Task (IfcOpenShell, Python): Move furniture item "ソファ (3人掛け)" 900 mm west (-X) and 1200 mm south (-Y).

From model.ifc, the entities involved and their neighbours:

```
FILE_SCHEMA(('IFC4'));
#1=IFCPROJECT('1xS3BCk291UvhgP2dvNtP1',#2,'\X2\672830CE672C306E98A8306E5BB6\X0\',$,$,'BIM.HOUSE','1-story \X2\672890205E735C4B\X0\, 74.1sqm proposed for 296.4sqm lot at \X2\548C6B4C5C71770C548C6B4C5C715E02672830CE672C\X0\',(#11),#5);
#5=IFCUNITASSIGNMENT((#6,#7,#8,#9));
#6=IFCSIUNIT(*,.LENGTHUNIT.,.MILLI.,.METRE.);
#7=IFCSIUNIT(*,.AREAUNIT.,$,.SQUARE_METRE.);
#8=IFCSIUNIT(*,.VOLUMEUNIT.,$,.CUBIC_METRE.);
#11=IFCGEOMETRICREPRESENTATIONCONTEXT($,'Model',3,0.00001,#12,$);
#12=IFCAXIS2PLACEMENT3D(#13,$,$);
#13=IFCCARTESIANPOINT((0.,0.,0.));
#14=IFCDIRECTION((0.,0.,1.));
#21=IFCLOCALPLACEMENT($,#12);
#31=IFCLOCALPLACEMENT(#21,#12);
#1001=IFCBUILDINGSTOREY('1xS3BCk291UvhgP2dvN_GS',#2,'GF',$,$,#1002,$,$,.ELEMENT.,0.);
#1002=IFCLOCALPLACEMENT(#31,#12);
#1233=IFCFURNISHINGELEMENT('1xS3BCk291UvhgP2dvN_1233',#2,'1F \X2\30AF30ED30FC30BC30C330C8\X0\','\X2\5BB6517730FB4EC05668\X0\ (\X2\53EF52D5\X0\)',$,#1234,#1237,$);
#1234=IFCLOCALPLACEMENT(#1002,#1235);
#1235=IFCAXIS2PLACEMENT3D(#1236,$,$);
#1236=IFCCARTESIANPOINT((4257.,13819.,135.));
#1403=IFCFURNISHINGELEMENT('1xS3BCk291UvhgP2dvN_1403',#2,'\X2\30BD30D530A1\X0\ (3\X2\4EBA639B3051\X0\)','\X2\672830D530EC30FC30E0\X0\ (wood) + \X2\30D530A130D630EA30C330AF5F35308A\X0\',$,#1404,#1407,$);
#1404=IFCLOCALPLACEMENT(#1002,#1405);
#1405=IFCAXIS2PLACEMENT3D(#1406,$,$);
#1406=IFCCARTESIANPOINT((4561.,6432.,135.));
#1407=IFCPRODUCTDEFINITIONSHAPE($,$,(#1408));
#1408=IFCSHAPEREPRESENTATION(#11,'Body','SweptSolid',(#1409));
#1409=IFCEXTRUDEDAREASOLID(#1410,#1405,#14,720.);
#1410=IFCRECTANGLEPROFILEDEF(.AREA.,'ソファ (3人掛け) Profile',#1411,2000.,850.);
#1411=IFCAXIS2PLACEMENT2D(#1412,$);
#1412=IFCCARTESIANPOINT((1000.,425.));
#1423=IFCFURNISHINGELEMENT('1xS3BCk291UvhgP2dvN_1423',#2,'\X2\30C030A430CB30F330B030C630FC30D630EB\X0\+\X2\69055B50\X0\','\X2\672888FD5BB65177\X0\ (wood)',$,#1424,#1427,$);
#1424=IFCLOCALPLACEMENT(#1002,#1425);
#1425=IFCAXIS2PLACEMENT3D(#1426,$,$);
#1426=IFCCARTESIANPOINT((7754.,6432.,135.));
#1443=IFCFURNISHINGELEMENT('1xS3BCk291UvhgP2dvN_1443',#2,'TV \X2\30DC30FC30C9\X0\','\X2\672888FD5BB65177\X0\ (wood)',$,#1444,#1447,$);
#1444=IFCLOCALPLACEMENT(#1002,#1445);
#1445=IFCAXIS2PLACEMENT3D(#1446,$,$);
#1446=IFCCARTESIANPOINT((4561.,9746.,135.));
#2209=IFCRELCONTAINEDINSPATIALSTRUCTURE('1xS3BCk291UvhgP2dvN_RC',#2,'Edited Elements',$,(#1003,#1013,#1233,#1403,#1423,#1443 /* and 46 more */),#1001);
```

```python
import ifcopenshell
import ifcopenshell.api.geometry
import ifcopenshell.util.placement
import ifcopenshell.util.unit

model = ifcopenshell.open("model.ifc")
unit_scale = ifcopenshell.util.unit.calculate_unit_scale(model)

item = model.by_id(1403)
matrix = ifcopenshell.util.placement.get_local_placement(item.ObjectPlacement)
matrix[0, 3] -= 0.9 / unit_scale
matrix[1, 3] -= 1.2 / unit_scale
ifcopenshell.api.geometry.edit_object_placement(model, product=item, matrix=matrix, is_si=False)

print(ifcopenshell.util.placement.get_local_placement(item.ObjectPlacement).round(3) + 0.0)

model.write("model_updated.ifc")
```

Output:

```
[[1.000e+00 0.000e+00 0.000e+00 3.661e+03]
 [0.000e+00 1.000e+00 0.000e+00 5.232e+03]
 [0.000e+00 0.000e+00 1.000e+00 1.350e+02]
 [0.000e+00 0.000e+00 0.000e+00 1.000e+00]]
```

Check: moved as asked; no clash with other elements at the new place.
